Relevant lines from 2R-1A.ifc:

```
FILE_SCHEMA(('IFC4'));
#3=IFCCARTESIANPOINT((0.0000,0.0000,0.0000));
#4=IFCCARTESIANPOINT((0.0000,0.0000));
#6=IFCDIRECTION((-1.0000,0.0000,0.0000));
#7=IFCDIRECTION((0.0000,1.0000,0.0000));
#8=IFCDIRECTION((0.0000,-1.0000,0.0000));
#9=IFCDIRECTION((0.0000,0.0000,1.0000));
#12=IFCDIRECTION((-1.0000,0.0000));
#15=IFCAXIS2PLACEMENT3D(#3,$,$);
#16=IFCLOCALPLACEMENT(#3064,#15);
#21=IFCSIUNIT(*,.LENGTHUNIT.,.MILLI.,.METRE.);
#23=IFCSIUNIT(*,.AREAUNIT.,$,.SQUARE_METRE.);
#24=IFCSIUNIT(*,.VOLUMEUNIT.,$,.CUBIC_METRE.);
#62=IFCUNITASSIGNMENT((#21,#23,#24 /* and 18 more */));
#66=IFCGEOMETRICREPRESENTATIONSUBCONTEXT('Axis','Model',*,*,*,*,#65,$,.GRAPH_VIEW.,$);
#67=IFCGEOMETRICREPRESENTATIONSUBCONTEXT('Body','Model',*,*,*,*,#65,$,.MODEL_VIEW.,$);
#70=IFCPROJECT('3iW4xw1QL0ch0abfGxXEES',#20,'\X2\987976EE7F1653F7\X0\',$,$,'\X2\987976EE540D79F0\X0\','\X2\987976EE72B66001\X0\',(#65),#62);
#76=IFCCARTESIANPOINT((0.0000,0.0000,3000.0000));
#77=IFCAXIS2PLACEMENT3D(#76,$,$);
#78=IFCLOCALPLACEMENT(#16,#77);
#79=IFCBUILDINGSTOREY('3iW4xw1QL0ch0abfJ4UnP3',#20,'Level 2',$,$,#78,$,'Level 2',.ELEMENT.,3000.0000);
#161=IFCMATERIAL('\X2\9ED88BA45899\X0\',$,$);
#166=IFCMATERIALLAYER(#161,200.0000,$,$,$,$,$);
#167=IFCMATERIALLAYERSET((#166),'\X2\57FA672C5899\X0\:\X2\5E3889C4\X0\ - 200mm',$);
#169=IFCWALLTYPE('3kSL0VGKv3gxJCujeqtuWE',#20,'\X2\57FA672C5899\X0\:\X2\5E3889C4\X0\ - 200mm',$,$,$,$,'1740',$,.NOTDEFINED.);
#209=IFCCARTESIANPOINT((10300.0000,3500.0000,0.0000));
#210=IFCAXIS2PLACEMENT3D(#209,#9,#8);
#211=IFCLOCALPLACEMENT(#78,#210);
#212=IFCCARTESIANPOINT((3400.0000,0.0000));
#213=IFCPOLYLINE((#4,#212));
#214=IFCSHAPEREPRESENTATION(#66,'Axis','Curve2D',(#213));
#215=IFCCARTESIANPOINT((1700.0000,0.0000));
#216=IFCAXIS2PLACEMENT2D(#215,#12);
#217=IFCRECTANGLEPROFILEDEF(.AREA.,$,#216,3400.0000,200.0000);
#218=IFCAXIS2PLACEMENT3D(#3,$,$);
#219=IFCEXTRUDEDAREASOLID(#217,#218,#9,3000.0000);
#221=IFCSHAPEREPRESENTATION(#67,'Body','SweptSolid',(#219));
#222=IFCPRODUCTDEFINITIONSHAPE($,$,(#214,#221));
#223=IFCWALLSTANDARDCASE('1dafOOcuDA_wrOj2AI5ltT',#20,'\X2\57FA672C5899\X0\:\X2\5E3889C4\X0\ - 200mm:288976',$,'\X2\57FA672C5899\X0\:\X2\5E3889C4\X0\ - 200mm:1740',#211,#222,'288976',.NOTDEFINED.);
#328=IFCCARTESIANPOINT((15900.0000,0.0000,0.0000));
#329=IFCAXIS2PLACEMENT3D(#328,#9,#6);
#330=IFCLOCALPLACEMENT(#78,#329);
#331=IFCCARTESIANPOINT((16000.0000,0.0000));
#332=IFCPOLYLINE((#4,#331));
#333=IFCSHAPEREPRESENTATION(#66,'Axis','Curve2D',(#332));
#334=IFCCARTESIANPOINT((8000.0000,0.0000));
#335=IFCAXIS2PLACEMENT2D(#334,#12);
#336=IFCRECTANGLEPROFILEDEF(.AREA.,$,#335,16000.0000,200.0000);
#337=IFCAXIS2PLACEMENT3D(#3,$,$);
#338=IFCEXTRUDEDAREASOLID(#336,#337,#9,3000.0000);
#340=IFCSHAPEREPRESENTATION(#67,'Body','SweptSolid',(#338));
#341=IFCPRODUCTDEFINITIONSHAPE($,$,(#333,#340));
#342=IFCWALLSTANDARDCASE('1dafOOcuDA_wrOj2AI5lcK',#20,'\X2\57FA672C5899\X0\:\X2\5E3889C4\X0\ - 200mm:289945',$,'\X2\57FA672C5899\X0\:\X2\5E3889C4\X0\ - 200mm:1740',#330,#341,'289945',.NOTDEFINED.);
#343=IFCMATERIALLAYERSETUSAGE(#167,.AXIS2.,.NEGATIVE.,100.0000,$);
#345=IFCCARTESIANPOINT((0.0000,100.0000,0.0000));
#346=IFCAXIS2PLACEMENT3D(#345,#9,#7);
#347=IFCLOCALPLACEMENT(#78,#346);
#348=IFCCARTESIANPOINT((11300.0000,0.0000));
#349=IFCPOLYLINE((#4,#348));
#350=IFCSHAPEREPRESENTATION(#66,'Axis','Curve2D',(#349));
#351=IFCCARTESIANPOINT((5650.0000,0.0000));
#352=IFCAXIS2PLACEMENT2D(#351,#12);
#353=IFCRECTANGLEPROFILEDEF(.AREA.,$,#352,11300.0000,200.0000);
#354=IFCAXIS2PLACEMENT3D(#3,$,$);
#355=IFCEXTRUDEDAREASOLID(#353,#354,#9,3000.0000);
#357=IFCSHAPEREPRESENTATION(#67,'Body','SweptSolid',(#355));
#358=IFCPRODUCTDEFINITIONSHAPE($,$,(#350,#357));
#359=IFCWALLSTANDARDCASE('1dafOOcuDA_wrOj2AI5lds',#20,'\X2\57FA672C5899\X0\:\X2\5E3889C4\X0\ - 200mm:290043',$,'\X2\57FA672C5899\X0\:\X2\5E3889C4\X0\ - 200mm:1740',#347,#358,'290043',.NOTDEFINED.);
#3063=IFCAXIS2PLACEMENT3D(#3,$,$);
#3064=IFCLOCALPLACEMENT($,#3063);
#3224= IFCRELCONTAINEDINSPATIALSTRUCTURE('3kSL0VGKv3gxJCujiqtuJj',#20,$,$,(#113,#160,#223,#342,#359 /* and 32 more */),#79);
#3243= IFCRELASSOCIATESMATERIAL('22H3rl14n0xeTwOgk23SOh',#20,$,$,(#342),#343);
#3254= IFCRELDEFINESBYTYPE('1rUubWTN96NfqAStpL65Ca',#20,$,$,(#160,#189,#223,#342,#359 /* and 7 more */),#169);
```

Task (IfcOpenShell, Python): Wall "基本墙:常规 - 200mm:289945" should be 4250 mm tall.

```python
import ifcopenshell
import ifcopenshell.geom
import ifcopenshell.util.representation
import ifcopenshell.util.shape

model = ifcopenshell.open("2R-1A.ifc")
settings = ifcopenshell.geom.settings()


def volume(element):
    """Net volume in cubic metres, openings subtracted."""
    shape = ifcopenshell.geom.create_shape(settings, element)
    return ifcopenshell.util.shape.get_volume(shape.geometry)


wall = model.by_guid("1dafOOcuDA_wrOj2AI5lcK")
before = volume(wall)

body = ifcopenshell.util.representation.get_representation(wall, "Model", "Body")
solid = body.Items[0]
old_height = solid.Depth
solid.Depth = 4250.0
after = volume(wall)

print(f"height {old_height:g} -> {solid.Depth:g}, volume {before:.3f} -> {after:.3f} m3")

model.write("2R-1A-out.ifc")
```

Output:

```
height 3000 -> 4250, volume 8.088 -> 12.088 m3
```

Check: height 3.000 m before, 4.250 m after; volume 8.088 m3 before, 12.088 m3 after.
